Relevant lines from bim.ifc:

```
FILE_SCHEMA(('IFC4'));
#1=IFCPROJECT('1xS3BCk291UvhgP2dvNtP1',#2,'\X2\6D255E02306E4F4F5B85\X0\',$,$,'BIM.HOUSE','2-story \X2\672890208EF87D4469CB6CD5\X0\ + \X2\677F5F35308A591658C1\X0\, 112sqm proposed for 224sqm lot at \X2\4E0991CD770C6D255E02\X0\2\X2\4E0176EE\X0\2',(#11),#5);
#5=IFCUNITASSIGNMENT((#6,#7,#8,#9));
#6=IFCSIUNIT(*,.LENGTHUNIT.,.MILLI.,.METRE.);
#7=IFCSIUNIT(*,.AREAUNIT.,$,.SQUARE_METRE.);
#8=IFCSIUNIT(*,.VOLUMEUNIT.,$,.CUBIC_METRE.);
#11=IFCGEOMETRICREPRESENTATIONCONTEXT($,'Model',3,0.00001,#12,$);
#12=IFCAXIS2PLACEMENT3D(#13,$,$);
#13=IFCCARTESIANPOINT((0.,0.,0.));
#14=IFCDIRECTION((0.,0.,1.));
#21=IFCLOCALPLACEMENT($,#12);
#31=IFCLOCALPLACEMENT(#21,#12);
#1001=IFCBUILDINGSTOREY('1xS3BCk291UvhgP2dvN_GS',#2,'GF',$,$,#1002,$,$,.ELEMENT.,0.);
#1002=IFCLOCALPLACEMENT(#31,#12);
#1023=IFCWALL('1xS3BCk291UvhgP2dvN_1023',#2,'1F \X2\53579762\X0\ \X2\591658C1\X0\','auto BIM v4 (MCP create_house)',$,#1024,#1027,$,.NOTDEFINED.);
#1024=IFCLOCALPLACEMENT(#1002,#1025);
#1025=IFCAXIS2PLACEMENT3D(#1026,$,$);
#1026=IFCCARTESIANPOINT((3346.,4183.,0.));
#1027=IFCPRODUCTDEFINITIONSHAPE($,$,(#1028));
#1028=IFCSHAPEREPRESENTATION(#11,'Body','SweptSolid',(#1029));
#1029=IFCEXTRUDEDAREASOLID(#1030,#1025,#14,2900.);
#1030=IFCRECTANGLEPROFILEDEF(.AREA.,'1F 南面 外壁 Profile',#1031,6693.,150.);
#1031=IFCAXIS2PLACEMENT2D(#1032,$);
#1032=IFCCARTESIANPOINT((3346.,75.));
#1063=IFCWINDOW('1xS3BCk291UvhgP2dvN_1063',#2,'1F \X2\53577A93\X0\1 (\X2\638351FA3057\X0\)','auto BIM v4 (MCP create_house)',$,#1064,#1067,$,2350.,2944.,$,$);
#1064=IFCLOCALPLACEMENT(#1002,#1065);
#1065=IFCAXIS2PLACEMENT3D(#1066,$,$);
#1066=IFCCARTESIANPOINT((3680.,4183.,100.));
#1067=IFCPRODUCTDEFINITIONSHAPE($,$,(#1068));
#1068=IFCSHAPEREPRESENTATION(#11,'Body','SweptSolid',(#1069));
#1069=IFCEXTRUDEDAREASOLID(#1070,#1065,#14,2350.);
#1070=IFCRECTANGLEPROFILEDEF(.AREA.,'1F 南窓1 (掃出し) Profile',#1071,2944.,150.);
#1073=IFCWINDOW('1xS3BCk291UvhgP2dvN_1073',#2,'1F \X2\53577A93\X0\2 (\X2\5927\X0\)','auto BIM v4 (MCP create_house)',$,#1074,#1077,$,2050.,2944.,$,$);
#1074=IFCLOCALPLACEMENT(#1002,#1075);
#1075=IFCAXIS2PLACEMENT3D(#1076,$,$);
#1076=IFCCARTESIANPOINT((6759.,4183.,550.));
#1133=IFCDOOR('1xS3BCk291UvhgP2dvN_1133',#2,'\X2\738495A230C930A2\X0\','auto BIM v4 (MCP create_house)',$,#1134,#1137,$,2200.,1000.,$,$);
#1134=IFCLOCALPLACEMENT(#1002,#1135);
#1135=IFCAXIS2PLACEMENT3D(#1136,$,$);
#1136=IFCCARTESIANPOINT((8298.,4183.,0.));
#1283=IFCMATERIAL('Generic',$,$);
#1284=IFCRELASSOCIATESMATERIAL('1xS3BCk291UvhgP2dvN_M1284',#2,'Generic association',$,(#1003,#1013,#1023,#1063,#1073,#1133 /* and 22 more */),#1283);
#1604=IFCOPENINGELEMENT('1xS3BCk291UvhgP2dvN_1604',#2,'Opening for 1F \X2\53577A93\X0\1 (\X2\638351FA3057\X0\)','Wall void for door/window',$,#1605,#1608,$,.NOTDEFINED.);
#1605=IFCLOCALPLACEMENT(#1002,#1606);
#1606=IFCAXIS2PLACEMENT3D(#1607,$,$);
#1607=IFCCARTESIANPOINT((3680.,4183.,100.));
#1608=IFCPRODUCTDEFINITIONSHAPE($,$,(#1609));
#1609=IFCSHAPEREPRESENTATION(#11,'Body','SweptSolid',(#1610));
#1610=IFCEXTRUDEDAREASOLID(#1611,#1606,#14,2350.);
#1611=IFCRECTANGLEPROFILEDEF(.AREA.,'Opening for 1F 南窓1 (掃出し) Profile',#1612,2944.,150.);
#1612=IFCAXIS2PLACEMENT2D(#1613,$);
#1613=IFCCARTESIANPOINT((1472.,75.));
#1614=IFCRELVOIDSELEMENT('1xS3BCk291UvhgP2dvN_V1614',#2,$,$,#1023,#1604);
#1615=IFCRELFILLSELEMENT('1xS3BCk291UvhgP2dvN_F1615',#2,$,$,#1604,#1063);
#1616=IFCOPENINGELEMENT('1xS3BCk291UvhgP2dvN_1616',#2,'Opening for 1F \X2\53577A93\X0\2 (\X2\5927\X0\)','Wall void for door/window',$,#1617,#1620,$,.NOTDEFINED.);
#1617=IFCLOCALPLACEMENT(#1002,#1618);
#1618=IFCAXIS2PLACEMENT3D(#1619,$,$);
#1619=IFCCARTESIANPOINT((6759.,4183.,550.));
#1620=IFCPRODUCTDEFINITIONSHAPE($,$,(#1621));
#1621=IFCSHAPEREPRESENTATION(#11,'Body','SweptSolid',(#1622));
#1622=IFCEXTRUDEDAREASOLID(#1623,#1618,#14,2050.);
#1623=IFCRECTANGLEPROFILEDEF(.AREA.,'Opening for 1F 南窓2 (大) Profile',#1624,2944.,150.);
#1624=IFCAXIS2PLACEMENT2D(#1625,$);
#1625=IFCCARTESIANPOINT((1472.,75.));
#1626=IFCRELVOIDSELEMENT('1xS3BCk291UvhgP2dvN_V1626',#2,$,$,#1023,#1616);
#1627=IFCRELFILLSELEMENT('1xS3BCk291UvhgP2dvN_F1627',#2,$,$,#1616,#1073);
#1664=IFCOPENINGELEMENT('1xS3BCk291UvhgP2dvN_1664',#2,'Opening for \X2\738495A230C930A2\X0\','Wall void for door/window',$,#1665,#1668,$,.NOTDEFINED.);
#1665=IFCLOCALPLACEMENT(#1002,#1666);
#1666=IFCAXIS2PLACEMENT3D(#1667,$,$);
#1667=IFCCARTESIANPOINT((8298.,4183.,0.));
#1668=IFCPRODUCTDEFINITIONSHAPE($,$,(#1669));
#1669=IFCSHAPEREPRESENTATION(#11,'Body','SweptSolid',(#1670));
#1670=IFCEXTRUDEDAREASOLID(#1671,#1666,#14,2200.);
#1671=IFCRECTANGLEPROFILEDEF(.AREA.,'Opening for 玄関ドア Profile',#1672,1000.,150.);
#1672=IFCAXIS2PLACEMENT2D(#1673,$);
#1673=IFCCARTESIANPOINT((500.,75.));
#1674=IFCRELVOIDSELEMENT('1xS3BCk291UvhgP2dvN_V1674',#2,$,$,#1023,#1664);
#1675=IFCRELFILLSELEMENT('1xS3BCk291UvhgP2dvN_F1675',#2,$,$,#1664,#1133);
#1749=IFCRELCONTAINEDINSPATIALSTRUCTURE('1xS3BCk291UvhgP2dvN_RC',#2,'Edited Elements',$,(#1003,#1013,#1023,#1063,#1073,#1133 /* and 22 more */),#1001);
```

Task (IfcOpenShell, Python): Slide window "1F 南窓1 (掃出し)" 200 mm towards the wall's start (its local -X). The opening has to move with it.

```python
import ifcopenshell
import ifcopenshell.api.geometry
import ifcopenshell.util.placement

model = ifcopenshell.open("bim.ifc")

window = model.by_guid("1xS3BCk291UvhgP2dvN_1063")
opening = window.FillsVoids[0].RelatingOpeningElement
wall = opening.VoidsElements[0].RelatingBuildingElement

wall_matrix = ifcopenshell.util.placement.get_local_placement(wall.ObjectPlacement)
shift = wall_matrix[:3, 0] * -200.0
before = ifcopenshell.util.placement.get_local_placement(window.ObjectPlacement)[:3, 3].copy()

# The window is not placed relative to its opening, so move both.
for product in (opening, window):
    matrix = ifcopenshell.util.placement.get_local_placement(product.ObjectPlacement)
    matrix[:3, 3] += shift
    ifcopenshell.api.geometry.edit_object_placement(model, product=product, matrix=matrix, is_si=False)

after = ifcopenshell.util.placement.get_local_placement(window.ObjectPlacement)[:3, 3]
print("window moved by", (after - before).round(3) + 0.0)

model.write("bim_rev.ifc")
```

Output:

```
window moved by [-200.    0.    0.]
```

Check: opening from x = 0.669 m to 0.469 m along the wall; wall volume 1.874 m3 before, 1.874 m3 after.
